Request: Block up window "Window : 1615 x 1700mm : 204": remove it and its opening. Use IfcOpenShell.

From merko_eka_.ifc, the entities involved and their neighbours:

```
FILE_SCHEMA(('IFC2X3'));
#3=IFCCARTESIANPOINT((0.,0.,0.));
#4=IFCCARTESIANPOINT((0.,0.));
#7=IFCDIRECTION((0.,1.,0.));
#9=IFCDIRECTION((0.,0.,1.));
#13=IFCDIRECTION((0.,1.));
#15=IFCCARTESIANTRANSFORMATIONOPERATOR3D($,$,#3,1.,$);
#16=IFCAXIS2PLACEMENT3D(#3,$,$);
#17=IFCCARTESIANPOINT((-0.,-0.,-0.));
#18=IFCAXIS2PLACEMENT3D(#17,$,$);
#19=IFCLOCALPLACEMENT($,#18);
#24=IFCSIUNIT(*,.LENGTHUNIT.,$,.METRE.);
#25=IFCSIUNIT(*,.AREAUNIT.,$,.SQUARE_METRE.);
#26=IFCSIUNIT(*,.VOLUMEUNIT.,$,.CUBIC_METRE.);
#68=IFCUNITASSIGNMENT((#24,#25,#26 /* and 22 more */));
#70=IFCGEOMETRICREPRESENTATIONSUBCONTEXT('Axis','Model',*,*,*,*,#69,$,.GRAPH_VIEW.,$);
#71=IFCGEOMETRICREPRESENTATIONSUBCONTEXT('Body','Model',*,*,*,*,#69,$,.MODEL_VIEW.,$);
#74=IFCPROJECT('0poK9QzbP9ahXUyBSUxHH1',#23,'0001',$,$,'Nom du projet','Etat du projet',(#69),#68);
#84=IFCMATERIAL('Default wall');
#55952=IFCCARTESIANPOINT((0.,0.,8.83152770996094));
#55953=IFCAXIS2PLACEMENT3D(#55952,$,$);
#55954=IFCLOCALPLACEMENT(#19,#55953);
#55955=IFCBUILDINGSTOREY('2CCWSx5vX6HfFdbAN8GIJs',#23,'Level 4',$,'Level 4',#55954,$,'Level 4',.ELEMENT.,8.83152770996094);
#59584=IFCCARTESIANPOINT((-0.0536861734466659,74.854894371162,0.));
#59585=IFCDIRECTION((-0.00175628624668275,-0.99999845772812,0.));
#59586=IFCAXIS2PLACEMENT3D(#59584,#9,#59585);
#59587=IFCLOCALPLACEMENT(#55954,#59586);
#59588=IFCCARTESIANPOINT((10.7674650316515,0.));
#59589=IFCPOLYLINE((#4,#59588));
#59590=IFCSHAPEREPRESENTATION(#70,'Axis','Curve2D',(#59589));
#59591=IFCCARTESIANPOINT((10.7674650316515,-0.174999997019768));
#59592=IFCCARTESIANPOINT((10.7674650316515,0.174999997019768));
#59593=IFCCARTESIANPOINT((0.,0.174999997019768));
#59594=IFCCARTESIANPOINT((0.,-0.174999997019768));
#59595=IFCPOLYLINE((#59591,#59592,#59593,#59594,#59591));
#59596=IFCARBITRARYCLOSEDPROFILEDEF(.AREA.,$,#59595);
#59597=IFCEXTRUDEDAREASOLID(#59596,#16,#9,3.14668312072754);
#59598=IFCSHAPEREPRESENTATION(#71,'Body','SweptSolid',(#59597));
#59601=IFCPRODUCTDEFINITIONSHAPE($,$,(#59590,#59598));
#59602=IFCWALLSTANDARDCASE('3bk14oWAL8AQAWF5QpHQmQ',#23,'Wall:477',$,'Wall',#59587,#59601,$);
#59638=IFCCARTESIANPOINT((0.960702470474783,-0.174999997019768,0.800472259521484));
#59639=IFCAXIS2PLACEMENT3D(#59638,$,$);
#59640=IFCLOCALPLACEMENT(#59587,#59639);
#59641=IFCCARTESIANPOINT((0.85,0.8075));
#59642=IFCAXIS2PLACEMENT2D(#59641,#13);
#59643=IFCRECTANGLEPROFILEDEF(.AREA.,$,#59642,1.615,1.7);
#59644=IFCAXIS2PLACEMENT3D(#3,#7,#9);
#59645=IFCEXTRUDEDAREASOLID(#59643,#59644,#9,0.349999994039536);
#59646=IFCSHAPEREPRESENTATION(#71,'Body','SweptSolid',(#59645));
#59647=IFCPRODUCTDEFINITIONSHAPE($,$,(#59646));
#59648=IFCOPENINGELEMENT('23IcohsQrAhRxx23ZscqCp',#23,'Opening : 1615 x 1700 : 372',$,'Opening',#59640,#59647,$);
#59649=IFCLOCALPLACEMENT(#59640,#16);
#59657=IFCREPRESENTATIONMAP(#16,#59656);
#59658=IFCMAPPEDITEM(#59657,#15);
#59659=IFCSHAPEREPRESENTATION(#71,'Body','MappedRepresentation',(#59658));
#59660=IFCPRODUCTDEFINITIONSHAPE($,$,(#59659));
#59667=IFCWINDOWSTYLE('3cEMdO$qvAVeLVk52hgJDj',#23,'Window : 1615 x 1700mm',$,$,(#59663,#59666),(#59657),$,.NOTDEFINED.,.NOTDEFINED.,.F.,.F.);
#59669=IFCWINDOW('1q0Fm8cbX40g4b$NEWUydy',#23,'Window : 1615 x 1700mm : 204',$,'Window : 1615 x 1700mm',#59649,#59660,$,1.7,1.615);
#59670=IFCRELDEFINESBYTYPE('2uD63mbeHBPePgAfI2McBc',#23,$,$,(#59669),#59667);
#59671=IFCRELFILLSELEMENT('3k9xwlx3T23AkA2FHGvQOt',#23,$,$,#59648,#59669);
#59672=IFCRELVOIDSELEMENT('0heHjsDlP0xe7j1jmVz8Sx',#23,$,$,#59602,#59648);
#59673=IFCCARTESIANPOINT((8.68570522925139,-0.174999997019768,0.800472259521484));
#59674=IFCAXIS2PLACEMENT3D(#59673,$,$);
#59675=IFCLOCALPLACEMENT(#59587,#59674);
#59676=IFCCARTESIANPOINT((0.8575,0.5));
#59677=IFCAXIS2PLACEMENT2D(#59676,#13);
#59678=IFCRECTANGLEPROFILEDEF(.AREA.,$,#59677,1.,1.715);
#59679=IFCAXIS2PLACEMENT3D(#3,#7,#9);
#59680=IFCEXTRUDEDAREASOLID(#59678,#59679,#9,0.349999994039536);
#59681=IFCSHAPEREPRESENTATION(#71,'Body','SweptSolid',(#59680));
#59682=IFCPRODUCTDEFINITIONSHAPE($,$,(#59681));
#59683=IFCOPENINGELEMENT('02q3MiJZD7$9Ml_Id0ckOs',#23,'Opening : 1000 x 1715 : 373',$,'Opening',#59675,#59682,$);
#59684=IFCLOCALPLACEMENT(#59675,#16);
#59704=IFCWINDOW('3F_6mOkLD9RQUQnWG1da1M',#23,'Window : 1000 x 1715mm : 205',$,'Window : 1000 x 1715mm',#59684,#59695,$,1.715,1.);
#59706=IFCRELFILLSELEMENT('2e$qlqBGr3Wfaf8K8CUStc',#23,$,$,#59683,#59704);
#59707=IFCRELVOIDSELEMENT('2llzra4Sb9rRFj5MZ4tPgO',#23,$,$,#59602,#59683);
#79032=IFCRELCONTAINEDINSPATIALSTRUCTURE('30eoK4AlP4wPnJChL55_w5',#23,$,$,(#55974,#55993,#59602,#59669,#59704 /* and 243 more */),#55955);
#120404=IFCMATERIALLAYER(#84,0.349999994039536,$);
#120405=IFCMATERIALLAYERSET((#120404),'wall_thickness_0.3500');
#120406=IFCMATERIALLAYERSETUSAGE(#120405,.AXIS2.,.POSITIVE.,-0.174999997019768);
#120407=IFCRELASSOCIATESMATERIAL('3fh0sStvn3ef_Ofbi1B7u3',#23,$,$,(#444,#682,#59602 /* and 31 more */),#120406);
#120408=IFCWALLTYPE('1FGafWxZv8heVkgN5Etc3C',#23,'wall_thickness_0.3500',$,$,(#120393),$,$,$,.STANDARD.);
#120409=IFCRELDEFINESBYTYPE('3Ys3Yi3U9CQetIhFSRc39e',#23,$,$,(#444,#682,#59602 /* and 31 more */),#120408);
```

```python
import ifcopenshell
import ifcopenshell.api.feature
import ifcopenshell.api.root
import ifcopenshell.geom
import ifcopenshell.util.shape

model = ifcopenshell.open("merko_eka_.ifc")
settings = ifcopenshell.geom.settings()


def volume(element):
    """Net volume in cubic metres, openings subtracted."""
    shape = ifcopenshell.geom.create_shape(settings, element)
    return ifcopenshell.util.shape.get_volume(shape.geometry)


window = model.by_id(59669)
opening = window.FillsVoids[0].RelatingOpeningElement
wall = opening.VoidsElements[0].RelatingBuildingElement
before = volume(wall)

ifcopenshell.api.root.remove_product(model, product=window)
ifcopenshell.api.feature.remove_feature(model, feature=opening)

after = volume(wall)

print(f"wall volume {before:.3f} -> {after:.3f} m3")

model.write("merko_eka__v2.ifc")
```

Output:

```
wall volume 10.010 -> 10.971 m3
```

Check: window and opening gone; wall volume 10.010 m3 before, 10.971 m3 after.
